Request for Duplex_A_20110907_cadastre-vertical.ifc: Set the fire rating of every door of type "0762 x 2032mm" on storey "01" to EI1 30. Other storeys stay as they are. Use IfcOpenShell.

First a look at what the model holds.

```python
import ifcopenshell
import ifcopenshell.util.element

model = ifcopenshell.open("Duplex_A_20110907_cadastre-vertical.ifc")
print(model.schema)
storey = next(s for s in model.by_type("IfcBuildingStorey") if s.Name == "01")
doors = [e for e in ifcopenshell.util.element.get_decomposition(storey) if e.is_a("IfcDoor")]
seen = {}
for e in doors:
    element_type = ifcopenshell.util.element.get_type(e)
    key = (element_type.Name if element_type != e and element_type else None, ifcopenshell.util.element.get_pset(e, "Pset_DoorCommon", "FireRating"))
    seen[key] = seen.get(key, 0) + 1
for (name, value), count in sorted(seen.items(), key=str):
    print(count, "x", name, "|", value)
```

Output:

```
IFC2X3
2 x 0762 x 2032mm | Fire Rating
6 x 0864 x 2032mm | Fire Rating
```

```python
import ifcopenshell
import ifcopenshell.api.pset
import ifcopenshell.util.element

model = ifcopenshell.open("Duplex_A_20110907_cadastre-vertical.ifc")

storey = next(s for s in model.by_type("IfcBuildingStorey") if s.Name == "01")
doors = [e for e in ifcopenshell.util.element.get_decomposition(storey) if e.is_a("IfcDoor")]

count = 0
for e in doors:
    element_type = ifcopenshell.util.element.get_type(e)
    if element_type in (None, e) or element_type.Name != "0762 x 2032mm":
        continue
    # add_pset returns the element's existing set when there is one.
    pset = ifcopenshell.api.pset.add_pset(model, product=e, name="Pset_DoorCommon")
    ifcopenshell.api.pset.edit_pset(model, pset=pset, properties={"FireRating": "EI1 30"})
    count += 1

print(count, "doors updated")

model.write("Duplex_A_20110907_cadastre-vertical_updated.ifc")
```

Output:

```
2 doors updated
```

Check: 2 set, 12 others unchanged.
